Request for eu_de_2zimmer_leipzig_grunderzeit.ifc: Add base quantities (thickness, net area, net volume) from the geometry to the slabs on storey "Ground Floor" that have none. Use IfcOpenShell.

First a look at what the model holds.

```python
import ifcopenshell
import ifcopenshell.util.element
import ifcopenshell.util.unit

model = ifcopenshell.open("eu_de_2zimmer_leipzig_grunderzeit.ifc")
print(model.schema)
for unit_type in ("LENGTHUNIT", "AREAUNIT", "VOLUMEUNIT"):
    print(unit_type, ifcopenshell.util.unit.calculate_unit_scale(model, unit_type))
storey = next(s for s in model.by_type("IfcBuildingStorey") if s.Name == "Ground Floor")
slabs = [e for e in ifcopenshell.util.element.get_decomposition(storey) if e.is_a("IfcSlab")]
for e in sorted(slabs, key=lambda e: e.id()):
    print(e.id(), e.is_a(), e.Name, list(ifcopenshell.util.element.get_psets(e, qtos_only=True)), sep=" | ")
```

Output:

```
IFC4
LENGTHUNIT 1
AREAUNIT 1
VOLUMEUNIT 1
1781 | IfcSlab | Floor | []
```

```python
import ifcopenshell
import ifcopenshell.api.pset
import ifcopenshell.geom
import ifcopenshell.util.element
import ifcopenshell.util.shape
import ifcopenshell.util.unit

model = ifcopenshell.open("eu_de_2zimmer_leipzig_grunderzeit.ifc")
unit_scale = ifcopenshell.util.unit.calculate_unit_scale(model)
area_scale = ifcopenshell.util.unit.calculate_unit_scale(model, "AREAUNIT")
volume_scale = ifcopenshell.util.unit.calculate_unit_scale(model, "VOLUMEUNIT")
settings = ifcopenshell.geom.settings()

storey = next(s for s in model.by_type("IfcBuildingStorey") if s.Name == "Ground Floor")
slabs = [e for e in ifcopenshell.util.element.get_decomposition(storey) if e.is_a("IfcSlab")]

for e in sorted(slabs, key=lambda e: e.id()):
    if ifcopenshell.util.element.get_psets(e, qtos_only=True, should_inherit=False):
        continue
    # Geometry comes back in metres, in the element's own axes.
    shape = ifcopenshell.geom.create_shape(settings, e)
    values = {
        "Width": ifcopenshell.util.shape.get_z(shape.geometry) / unit_scale,
        "NetArea": ifcopenshell.util.shape.get_footprint_area(shape.geometry) / area_scale,
        "NetVolume": ifcopenshell.util.shape.get_volume(shape.geometry) / volume_scale,
    }
    qto = ifcopenshell.api.pset.add_qto(model, product=e, name="Qto_SlabBaseQuantities")
    ifcopenshell.api.pset.edit_qto(model, qto=qto, properties=values)
    print(e.id(), {k: round(v, 3) for k, v in values.items()})

model.write("eu_de_2zimmer_leipzig_grunderzeit_v2.ifc")
```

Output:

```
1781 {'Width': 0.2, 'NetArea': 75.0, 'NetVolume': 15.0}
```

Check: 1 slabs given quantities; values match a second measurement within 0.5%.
